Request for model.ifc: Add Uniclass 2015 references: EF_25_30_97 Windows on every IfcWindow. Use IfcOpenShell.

First a look at what the model holds.

```python
import ifcopenshell

model = ifcopenshell.open("model.ifc")
print(model.schema)
print("classifications:", [c.Name for c in model.by_type("IfcClassification")])
for ifc_class in ("IfcDoor", "IfcRoof", "IfcStair", "IfcWall", "IfcWindow"):
    print(ifc_class, len(model.by_type(ifc_class)))
```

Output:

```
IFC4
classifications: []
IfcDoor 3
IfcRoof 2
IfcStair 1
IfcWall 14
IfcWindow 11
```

```python
import ifcopenshell
import ifcopenshell.api.classification

model = ifcopenshell.open("model.ifc")

system = ifcopenshell.api.classification.add_classification(model, classification="Uniclass 2015")

codes = {
    "IfcWindow": ("EF_25_30_97", "Windows"),
}
for ifc_class, (code, name) in codes.items():
    products = model.by_type(ifc_class)
    ifcopenshell.api.classification.add_reference(
        model, products=products, classification=system, identification=code, name=name
    )
    print(code, len(products))

model.write("model_updated.ifc")
```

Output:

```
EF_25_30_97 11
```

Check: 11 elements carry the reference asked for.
